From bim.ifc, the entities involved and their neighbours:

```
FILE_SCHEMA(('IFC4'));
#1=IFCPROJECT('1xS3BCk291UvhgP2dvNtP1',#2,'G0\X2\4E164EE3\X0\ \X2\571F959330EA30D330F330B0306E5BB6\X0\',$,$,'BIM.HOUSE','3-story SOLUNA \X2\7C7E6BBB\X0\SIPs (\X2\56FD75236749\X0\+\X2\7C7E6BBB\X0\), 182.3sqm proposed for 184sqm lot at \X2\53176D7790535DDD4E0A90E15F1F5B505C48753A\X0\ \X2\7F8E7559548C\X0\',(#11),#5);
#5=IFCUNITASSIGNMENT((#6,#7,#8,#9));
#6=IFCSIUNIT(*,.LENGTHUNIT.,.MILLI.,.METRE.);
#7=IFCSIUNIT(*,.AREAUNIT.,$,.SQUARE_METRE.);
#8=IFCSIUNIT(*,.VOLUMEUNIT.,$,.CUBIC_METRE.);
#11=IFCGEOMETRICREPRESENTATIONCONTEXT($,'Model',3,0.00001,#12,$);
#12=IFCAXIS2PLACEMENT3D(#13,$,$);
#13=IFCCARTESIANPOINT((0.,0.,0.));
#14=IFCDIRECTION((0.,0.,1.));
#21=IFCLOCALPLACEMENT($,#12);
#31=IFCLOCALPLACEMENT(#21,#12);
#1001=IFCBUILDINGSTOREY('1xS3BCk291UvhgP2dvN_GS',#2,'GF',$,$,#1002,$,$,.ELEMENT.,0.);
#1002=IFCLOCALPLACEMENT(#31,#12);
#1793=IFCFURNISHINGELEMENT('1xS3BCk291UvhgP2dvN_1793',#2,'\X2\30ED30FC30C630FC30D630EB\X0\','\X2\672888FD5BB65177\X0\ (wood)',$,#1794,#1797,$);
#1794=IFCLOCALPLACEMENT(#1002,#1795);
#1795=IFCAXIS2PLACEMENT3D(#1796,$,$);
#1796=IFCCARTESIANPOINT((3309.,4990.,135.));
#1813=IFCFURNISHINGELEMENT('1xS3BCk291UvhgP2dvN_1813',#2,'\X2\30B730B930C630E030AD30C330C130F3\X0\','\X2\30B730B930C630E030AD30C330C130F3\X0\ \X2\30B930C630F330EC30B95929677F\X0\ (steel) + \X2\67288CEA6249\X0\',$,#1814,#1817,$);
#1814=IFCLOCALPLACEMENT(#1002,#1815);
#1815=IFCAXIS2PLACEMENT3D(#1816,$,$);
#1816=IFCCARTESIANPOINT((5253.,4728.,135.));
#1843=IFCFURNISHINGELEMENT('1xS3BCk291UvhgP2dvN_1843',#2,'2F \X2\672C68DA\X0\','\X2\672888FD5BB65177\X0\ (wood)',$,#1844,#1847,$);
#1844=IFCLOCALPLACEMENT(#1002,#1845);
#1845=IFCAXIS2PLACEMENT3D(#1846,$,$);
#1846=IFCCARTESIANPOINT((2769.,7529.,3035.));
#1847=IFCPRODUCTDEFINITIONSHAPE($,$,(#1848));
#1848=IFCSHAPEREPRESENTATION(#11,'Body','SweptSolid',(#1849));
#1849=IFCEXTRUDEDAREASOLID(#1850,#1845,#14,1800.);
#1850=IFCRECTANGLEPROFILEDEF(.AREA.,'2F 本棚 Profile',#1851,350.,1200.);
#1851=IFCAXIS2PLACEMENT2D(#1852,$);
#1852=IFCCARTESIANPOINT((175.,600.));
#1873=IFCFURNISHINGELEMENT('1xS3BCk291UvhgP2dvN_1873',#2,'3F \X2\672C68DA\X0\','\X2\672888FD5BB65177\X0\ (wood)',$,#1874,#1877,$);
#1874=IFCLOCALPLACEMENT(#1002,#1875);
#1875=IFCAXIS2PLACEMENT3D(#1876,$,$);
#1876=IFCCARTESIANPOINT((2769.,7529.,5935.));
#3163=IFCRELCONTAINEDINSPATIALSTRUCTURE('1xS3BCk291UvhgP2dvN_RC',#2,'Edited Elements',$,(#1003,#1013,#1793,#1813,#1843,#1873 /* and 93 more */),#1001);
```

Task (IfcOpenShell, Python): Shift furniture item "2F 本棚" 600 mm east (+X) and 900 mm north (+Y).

```python
import ifcopenshell
import ifcopenshell.api.geometry
import ifcopenshell.util.placement

model = ifcopenshell.open("bim.ifc")

item = model.by_guid("1xS3BCk291UvhgP2dvN_1843")
matrix = ifcopenshell.util.placement.get_local_placement(item.ObjectPlacement)
matrix[0, 3] += 600.0
matrix[1, 3] += 900.0
ifcopenshell.api.geometry.edit_object_placement(model, product=item, matrix=matrix, is_si=False)

print(ifcopenshell.util.placement.get_local_placement(item.ObjectPlacement).round(3) + 0.0)

model.write("bim_rev.ifc")
```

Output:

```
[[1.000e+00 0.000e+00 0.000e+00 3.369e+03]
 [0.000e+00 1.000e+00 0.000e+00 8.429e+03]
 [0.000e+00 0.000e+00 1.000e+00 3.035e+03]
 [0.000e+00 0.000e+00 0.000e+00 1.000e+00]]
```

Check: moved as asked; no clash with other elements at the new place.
